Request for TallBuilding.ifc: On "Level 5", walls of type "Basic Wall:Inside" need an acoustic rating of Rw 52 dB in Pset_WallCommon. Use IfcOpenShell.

First a look at what the model holds.

```python
import ifcopenshell
import ifcopenshell.util.element

model = ifcopenshell.open("TallBuilding.ifc")
print(model.schema)
storey = next(s for s in model.by_type("IfcBuildingStorey") if s.Name == "Level 5")
walls = [e for e in ifcopenshell.util.element.get_decomposition(storey) if e.is_a("IfcWall")]
seen = {}
for e in walls:
    element_type = ifcopenshell.util.element.get_type(e)
    key = (element_type.Name if element_type != e and element_type else None, ifcopenshell.util.element.get_pset(e, "Pset_WallCommon", "AcousticRating"))
    seen[key] = seen.get(key, 0) + 1
for (name, value), count in sorted(seen.items(), key=str):
    print(count, "x", name, "|", value)
```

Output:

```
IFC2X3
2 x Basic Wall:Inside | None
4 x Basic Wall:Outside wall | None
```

```python
import ifcopenshell
import ifcopenshell.api.pset
import ifcopenshell.util.element

model = ifcopenshell.open("TallBuilding.ifc")

storey = next(s for s in model.by_type("IfcBuildingStorey") if s.Name == "Level 5")
walls = [e for e in ifcopenshell.util.element.get_decomposition(storey) if e.is_a("IfcWall")]

count = 0
for e in walls:
    element_type = ifcopenshell.util.element.get_type(e)
    if element_type in (None, e) or element_type.Name != "Basic Wall:Inside":
        continue
    # add_pset returns the element's existing set when there is one.
    pset = ifcopenshell.api.pset.add_pset(model, product=e, name="Pset_WallCommon")
    ifcopenshell.api.pset.edit_pset(model, pset=pset, properties={"AcousticRating": "Rw 52 dB"})
    count += 1

print(count, "walls updated")

model.write("TallBuilding_edited.ifc")
```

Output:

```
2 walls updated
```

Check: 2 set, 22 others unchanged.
